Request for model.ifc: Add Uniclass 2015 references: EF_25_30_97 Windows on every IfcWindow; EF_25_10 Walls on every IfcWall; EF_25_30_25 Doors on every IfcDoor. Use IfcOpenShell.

First a look at what the model holds.

```python
import ifcopenshell

model = ifcopenshell.open("model.ifc")
print(model.schema)
print("classifications:", [c.Name for c in model.by_type("IfcClassification")])
for ifc_class in ("IfcDoor", "IfcRoof", "IfcStair", "IfcWall", "IfcWindow"):
    print(ifc_class, len(model.by_type(ifc_class)))
```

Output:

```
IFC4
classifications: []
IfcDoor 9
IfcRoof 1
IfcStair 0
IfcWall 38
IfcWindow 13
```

```python
import ifcopenshell
import ifcopenshell.api.classification

model = ifcopenshell.open("model.ifc")

system = ifcopenshell.api.classification.add_classification(model, classification="Uniclass 2015")

codes = {
    "IfcWindow": ("EF_25_30_97", "Windows"),
    "IfcWall": ("EF_25_10", "Walls"),
    "IfcDoor": ("EF_25_30_25", "Doors"),
}
for ifc_class, (code, name) in codes.items():
    products = model.by_type(ifc_class)
    ifcopenshell.api.classification.add_reference(
        model, products=products, classification=system, identification=code, name=name
    )
    print(code, len(products))

model.write("model_edited.ifc")
```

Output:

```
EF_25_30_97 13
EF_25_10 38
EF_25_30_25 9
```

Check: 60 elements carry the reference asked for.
